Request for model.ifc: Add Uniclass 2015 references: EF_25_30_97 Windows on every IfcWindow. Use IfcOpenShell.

First a look at what the model holds.

```python
import ifcopenshell

model = ifcopenshell.open("model.ifc")
print(model.schema)
print("classifications:", [c.Name for c in model.by_type("IfcClassification")])
for ifc_class in ("IfcDoor", "IfcRoof", "IfcStair", "IfcWall", "IfcWindow"):
    print(ifc_class, len(model.by_type(ifc_class)))
```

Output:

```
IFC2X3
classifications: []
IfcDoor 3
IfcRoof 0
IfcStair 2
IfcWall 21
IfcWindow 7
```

```python
import ifcopenshell
import ifcopenshell.api.classification

model = ifcopenshell.open("model.ifc")

# IFC2X3 requires Source and Edition and has no link from the project to the system.
system = model.create_entity("IfcClassification", Source="NBS", Edition="2015", Name="Uniclass 2015")

codes = {
    "IfcWindow": ("EF_25_30_97", "Windows"),
}
for ifc_class, (code, name) in codes.items():
    products = model.by_type(ifc_class)
    ifcopenshell.api.classification.add_reference(
        model, products=products, classification=system, identification=code, name=name
    )
    print(code, len(products))

model.write("model_v2.ifc")
```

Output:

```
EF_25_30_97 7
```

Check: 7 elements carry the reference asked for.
